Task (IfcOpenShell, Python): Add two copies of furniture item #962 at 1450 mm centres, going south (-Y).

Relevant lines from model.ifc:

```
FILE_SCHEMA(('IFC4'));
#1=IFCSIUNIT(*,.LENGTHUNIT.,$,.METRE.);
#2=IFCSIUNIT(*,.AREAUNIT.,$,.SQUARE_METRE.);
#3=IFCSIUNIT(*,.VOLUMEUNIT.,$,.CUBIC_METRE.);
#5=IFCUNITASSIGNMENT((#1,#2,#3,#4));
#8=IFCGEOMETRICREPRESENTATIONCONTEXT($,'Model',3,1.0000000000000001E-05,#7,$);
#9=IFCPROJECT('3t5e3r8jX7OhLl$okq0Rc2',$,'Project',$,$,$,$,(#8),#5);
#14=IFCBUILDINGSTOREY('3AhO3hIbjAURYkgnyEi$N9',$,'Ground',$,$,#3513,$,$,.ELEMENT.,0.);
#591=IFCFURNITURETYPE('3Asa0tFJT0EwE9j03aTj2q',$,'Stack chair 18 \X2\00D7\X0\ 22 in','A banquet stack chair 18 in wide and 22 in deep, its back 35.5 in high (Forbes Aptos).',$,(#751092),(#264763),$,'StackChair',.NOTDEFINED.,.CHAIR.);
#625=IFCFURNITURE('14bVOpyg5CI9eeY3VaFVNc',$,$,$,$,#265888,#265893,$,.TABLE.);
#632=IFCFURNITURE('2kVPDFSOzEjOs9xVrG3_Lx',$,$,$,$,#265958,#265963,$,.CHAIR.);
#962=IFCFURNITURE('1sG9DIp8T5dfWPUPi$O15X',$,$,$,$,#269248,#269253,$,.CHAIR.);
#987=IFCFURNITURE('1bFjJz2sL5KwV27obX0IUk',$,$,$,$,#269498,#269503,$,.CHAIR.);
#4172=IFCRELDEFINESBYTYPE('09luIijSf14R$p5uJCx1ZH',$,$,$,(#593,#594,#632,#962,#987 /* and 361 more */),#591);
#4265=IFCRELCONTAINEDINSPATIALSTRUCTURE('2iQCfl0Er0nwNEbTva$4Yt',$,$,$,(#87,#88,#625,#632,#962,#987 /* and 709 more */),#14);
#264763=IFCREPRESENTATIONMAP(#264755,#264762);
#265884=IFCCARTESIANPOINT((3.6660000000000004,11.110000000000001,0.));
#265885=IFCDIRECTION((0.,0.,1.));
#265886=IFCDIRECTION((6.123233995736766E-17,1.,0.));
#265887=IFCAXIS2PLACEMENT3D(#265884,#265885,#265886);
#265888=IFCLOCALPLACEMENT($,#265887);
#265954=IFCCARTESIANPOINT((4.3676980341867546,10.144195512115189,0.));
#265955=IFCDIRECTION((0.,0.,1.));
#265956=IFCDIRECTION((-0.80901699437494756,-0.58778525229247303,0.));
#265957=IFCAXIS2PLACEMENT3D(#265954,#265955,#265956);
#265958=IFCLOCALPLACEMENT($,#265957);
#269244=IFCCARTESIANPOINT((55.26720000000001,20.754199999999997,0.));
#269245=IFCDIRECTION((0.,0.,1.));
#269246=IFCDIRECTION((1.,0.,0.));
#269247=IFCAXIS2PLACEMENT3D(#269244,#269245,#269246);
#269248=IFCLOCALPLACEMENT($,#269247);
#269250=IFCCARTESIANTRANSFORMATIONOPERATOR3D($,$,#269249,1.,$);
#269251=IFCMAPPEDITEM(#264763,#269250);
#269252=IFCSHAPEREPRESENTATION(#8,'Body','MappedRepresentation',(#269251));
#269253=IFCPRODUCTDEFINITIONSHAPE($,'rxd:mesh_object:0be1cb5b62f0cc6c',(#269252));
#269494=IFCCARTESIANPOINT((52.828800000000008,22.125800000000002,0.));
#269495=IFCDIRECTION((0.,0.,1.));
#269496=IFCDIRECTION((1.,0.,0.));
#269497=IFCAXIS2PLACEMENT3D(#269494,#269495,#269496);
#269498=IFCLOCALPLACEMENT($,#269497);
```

```python
import numpy as np
import ifcopenshell
import ifcopenshell.api.geometry
import ifcopenshell.api.root
import ifcopenshell.util.element
import ifcopenshell.util.placement
import ifcopenshell.util.unit

model = ifcopenshell.open("model.ifc")
unit_scale = ifcopenshell.util.unit.calculate_unit_scale(model)

source = model.by_id(962)
base = ifcopenshell.util.placement.get_local_placement(source.ObjectPlacement)
step = np.array([0.0, -1.0, 0.0]) * 1.45 / unit_scale

for i in range(1, 3):
    copy = ifcopenshell.api.root.copy_class(model, product=source)
    copy.Representation = ifcopenshell.util.element.copy_deep(
        model, source.Representation, exclude=["IfcGeometricRepresentationContext", "IfcRepresentationMap"]
    )
    matrix = base.copy()
    matrix[:3, 3] += i * step
    print("added at", matrix[:3, 3].round(3) + 0.0)
    ifcopenshell.api.geometry.edit_object_placement(model, product=copy, matrix=matrix, is_si=False)

model.write("model_edited.ifc")
```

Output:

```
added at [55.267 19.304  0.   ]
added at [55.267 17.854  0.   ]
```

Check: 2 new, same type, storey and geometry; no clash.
